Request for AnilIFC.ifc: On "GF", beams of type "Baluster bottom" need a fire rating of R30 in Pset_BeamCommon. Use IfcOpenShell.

First a look at what the model holds.

```python
import ifcopenshell
import ifcopenshell.util.element

model = ifcopenshell.open("AnilIFC.ifc")
print(model.schema)
storey = next(s for s in model.by_type("IfcBuildingStorey") if s.Name == "GF")
beams = [e for e in ifcopenshell.util.element.get_decomposition(storey) if e.is_a("IfcBeam")]
seen = {}
for e in beams:
    element_type = ifcopenshell.util.element.get_type(e)
    key = (element_type.Name if element_type != e and element_type else None, ifcopenshell.util.element.get_pset(e, "Pset_BeamCommon", "FireRating"))
    seen[key] = seen.get(key, 0) + 1
for (name, value), count in sorted(seen.items(), key=str):
    print(count, "x", name, "|", value)
```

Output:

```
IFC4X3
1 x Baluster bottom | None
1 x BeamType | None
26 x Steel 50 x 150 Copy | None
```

```python
import ifcopenshell
import ifcopenshell.api.pset
import ifcopenshell.util.element

model = ifcopenshell.open("AnilIFC.ifc")

storey = next(s for s in model.by_type("IfcBuildingStorey") if s.Name == "GF")
beams = [e for e in ifcopenshell.util.element.get_decomposition(storey) if e.is_a("IfcBeam")]

count = 0
for e in beams:
    element_type = ifcopenshell.util.element.get_type(e)
    if element_type in (None, e) or element_type.Name != "Baluster bottom":
        continue
    # add_pset returns the element's existing set when there is one.
    pset = ifcopenshell.api.pset.add_pset(model, product=e, name="Pset_BeamCommon")
    ifcopenshell.api.pset.edit_pset(model, pset=pset, properties={"FireRating": "R30"})
    count += 1

print(count, "beams updated")

model.write("AnilIFC_updated.ifc")
```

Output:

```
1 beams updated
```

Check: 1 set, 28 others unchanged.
